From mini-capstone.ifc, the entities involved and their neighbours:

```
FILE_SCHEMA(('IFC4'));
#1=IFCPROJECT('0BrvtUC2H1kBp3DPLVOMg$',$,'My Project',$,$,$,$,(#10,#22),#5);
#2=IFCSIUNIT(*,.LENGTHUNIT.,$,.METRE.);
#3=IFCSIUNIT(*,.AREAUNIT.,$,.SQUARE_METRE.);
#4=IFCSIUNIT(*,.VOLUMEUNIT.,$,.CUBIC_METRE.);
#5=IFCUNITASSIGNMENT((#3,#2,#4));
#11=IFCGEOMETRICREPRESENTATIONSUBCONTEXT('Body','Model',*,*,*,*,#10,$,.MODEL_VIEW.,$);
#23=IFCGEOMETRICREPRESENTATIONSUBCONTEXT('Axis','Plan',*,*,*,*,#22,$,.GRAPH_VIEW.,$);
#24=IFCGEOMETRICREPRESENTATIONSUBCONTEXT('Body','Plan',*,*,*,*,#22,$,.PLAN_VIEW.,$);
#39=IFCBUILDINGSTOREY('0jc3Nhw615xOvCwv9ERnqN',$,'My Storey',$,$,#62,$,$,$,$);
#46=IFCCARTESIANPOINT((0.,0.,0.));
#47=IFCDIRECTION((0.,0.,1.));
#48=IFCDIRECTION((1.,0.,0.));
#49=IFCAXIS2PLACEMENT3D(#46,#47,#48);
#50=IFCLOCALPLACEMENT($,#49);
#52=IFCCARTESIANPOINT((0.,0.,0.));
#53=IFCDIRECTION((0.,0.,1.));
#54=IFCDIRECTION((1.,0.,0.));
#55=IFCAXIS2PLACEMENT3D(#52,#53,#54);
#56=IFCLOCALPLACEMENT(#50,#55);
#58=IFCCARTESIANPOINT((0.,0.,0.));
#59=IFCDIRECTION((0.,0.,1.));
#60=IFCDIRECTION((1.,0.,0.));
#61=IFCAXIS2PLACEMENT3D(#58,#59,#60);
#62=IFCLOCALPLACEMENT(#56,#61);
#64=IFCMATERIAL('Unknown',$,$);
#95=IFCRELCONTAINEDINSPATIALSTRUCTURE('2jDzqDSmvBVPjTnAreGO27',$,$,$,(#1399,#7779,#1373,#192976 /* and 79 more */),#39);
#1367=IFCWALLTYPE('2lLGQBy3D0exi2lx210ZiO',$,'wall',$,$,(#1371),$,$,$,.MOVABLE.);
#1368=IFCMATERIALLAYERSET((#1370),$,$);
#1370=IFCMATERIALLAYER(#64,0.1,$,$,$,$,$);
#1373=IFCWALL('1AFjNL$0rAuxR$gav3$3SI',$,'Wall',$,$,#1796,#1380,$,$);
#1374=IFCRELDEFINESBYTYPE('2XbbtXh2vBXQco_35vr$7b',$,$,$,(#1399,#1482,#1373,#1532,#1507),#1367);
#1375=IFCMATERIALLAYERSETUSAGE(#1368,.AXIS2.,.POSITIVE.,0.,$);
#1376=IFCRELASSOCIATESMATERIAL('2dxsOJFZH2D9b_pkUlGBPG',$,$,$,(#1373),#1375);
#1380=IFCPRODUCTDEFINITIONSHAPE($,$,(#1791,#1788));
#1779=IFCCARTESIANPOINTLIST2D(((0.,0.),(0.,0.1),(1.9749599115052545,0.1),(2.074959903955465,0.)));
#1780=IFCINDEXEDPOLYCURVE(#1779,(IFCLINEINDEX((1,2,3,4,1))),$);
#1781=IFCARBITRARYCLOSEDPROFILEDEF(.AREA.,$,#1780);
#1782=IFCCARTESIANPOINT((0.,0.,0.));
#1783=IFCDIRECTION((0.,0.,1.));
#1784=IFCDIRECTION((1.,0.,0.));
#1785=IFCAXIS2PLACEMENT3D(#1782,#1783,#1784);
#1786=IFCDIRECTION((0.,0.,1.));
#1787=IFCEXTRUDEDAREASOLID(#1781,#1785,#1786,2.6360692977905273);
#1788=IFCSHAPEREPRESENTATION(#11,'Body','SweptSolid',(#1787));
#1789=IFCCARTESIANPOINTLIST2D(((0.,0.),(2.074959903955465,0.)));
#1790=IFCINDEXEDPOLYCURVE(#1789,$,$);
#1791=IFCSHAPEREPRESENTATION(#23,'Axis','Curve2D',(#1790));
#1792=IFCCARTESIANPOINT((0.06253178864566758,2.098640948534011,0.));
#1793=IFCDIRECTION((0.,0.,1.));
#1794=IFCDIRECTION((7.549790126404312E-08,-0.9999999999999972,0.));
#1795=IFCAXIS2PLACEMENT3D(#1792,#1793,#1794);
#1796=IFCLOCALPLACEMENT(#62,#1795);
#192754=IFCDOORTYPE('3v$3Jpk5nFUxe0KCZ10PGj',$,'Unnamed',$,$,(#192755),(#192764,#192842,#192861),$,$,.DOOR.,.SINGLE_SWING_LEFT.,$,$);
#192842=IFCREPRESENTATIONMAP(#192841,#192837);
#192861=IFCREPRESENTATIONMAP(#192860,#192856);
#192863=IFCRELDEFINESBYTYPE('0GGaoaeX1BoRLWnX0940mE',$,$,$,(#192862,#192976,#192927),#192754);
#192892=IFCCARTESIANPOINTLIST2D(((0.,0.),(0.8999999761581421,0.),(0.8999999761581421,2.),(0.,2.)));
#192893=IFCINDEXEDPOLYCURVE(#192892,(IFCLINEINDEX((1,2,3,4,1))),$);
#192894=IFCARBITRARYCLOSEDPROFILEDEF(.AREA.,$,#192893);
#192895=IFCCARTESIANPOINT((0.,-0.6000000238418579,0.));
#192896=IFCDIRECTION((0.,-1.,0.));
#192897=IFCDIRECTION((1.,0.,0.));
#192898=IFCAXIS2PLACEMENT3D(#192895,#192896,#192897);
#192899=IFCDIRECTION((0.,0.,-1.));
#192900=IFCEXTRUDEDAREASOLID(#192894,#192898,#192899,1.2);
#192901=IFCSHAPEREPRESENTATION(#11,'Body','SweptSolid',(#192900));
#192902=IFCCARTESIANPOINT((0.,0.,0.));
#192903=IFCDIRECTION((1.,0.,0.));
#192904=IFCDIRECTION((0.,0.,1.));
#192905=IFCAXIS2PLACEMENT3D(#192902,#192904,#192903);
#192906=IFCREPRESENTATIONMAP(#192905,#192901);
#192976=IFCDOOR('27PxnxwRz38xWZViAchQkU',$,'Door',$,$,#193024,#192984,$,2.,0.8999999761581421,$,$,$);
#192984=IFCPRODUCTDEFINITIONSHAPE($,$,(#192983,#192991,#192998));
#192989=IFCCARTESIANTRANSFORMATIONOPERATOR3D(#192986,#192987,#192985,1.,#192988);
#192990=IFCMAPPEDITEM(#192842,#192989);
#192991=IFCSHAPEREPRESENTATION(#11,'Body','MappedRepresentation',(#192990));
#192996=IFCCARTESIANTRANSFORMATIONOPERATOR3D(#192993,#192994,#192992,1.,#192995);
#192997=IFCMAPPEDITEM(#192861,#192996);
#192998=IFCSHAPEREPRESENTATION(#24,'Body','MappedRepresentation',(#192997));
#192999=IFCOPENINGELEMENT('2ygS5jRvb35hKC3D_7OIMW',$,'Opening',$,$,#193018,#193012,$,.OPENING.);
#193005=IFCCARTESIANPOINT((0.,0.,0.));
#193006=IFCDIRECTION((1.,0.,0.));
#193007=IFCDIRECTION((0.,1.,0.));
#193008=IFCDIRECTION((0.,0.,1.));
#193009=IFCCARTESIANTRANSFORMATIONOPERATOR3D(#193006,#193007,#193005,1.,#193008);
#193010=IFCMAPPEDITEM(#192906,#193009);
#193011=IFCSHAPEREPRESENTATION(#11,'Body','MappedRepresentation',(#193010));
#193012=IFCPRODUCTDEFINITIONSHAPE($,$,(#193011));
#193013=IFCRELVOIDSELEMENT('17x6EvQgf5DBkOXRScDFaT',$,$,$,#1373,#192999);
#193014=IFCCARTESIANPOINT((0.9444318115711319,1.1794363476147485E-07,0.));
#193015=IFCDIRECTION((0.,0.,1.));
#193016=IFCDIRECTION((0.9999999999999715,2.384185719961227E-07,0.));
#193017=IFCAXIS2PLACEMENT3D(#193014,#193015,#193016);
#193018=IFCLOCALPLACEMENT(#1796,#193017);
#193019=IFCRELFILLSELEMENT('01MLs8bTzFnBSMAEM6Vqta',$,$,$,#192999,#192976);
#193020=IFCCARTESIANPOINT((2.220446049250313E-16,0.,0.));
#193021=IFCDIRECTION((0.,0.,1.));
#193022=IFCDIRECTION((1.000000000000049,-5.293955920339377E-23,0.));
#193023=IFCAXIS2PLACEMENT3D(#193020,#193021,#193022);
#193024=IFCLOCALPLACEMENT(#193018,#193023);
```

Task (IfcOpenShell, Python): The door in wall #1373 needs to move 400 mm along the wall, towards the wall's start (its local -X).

```python
import ifcopenshell
import ifcopenshell.api.geometry
import ifcopenshell.util.placement

model = ifcopenshell.open("mini-capstone.ifc")

door = model.by_guid("27PxnxwRz38xWZViAchQkU")
opening = door.FillsVoids[0].RelatingOpeningElement
wall = opening.VoidsElements[0].RelatingBuildingElement

wall_matrix = ifcopenshell.util.placement.get_local_placement(wall.ObjectPlacement)
shift = wall_matrix[:3, 0] * -0.4
before = ifcopenshell.util.placement.get_local_placement(door.ObjectPlacement)[:3, 3].copy()

# The door is placed relative to its opening, so it follows when the opening moves.
matrix = ifcopenshell.util.placement.get_local_placement(opening.ObjectPlacement)
matrix[:3, 3] += shift
ifcopenshell.api.geometry.edit_object_placement(
    model, product=opening, matrix=matrix, is_si=False, should_transform_children=True
)

after = ifcopenshell.util.placement.get_local_placement(door.ObjectPlacement)[:3, 3]
print("door moved by", (after - before).round(3) + 0.0)

model.write("mini-capstone-out.ifc")
```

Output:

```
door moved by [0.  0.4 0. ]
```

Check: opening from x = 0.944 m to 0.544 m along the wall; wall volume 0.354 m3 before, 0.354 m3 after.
